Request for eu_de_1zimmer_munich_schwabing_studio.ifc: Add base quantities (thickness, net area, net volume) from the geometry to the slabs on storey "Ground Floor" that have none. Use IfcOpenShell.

First a look at what the model holds.

```python
import ifcopenshell
import ifcopenshell.util.element
import ifcopenshell.util.unit

model = ifcopenshell.open("eu_de_1zimmer_munich_schwabing_studio.ifc")
print(model.schema)
for unit_type in ("LENGTHUNIT", "AREAUNIT", "VOLUMEUNIT"):
    print(unit_type, ifcopenshell.util.unit.calculate_unit_scale(model, unit_type))
storey = next(s for s in model.by_type("IfcBuildingStorey") if s.Name == "Ground Floor")
slabs = [e for e in ifcopenshell.util.element.get_decomposition(storey) if e.is_a("IfcSlab")]
for e in sorted(slabs, key=lambda e: e.id()):
    print(e.id(), e.is_a(), e.Name, list(ifcopenshell.util.element.get_psets(e, qtos_only=True)), sep=" | ")
```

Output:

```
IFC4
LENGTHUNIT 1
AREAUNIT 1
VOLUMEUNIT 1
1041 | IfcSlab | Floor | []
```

```python
import ifcopenshell
import ifcopenshell.api.pset
import ifcopenshell.geom
import ifcopenshell.util.element
import ifcopenshell.util.shape
import ifcopenshell.util.unit

model = ifcopenshell.open("eu_de_1zimmer_munich_schwabing_studio.ifc")
unit_scale = ifcopenshell.util.unit.calculate_unit_scale(model)
area_scale = ifcopenshell.util.unit.calculate_unit_scale(model, "AREAUNIT")
volume_scale = ifcopenshell.util.unit.calculate_unit_scale(model, "VOLUMEUNIT")
settings = ifcopenshell.geom.settings()

storey = next(s for s in model.by_type("IfcBuildingStorey") if s.Name == "Ground Floor")
slabs = [e for e in ifcopenshell.util.element.get_decomposition(storey) if e.is_a("IfcSlab")]

for e in sorted(slabs, key=lambda e: e.id()):
    if ifcopenshell.util.element.get_psets(e, qtos_only=True, should_inherit=False):
        continue
    # Geometry comes back in metres, in the element's own axes.
    shape = ifcopenshell.geom.create_shape(settings, e)
    values = {
        "Width": ifcopenshell.util.shape.get_z(shape.geometry) / unit_scale,
        "NetArea": ifcopenshell.util.shape.get_footprint_area(shape.geometry) / area_scale,
        "NetVolume": ifcopenshell.util.shape.get_volume(shape.geometry) / volume_scale,
    }
    qto = ifcopenshell.api.pset.add_qto(model, product=e, name="Qto_SlabBaseQuantities")
    ifcopenshell.api.pset.edit_qto(model, qto=qto, properties=values)
    print(e.id(), {k: round(v, 3) for k, v in values.items()})

model.write("eu_de_1zimmer_munich_schwabing_studio_updated.ifc")
```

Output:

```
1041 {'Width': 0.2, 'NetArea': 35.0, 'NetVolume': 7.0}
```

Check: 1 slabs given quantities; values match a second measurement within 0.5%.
